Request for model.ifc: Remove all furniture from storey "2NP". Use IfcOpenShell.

First a look at what the model holds.

```python
import ifcopenshell
import ifcopenshell.util.element

model = ifcopenshell.open("model.ifc")
print(model.schema)
storey = next(s for s in model.by_type("IfcBuildingStorey") if s.Name == "2NP")
furniture = [e for e in ifcopenshell.util.element.get_decomposition(storey) if e.is_a("IfcFurnishingElement")]
seen = {}
for e in furniture:
    element_type = ifcopenshell.util.element.get_type(e)
    name = element_type.Name if element_type not in (None, e) else None
    seen[name] = seen.get(name, 0) + 1
for name, count in sorted(seen.items(), key=str):
    print(count, "x", name)
```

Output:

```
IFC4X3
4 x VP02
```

```python
import ifcopenshell
import ifcopenshell.api.root
import ifcopenshell.util.element

model = ifcopenshell.open("model.ifc")

storey = next(s for s in model.by_type("IfcBuildingStorey") if s.Name == "2NP")
furniture = [e for e in ifcopenshell.util.element.get_decomposition(storey) if e.is_a("IfcFurnishingElement")]

for e in furniture:
    ifcopenshell.api.root.remove_product(model, product=e)
print(len(furniture), "removed")

model.write("model_edited.ifc")
```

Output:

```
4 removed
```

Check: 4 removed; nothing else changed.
